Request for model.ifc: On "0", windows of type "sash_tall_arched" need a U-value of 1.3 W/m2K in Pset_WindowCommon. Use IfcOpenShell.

First a look at what the model holds.

```python
import ifcopenshell
import ifcopenshell.util.element

model = ifcopenshell.open("model.ifc")
print(model.schema)
storey = next(s for s in model.by_type("IfcBuildingStorey") if s.Name == "0")
windows = [e for e in ifcopenshell.util.element.get_decomposition(storey) if e.is_a("IfcWindow")]
seen = {}
for e in windows:
    element_type = ifcopenshell.util.element.get_type(e)
    key = (element_type.Name if element_type != e and element_type else None, ifcopenshell.util.element.get_pset(e, "Pset_WindowCommon", "ThermalTransmittance"))
    seen[key] = seen.get(key, 0) + 1
for (name, value), count in sorted(seen.items(), key=str):
    print(count, "x", name, "|", value)
```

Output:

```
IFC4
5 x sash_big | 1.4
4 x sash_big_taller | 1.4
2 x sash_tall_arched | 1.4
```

```python
import ifcopenshell
import ifcopenshell.api.pset
import ifcopenshell.util.element

model = ifcopenshell.open("model.ifc")

storey = next(s for s in model.by_type("IfcBuildingStorey") if s.Name == "0")
windows = [e for e in ifcopenshell.util.element.get_decomposition(storey) if e.is_a("IfcWindow")]

count = 0
for e in windows:
    element_type = ifcopenshell.util.element.get_type(e)
    if element_type in (None, e) or element_type.Name != "sash_tall_arched":
        continue
    # add_pset returns the element's existing set when there is one.
    pset = ifcopenshell.api.pset.add_pset(model, product=e, name="Pset_WindowCommon")
    ifcopenshell.api.pset.edit_pset(model, pset=pset, properties={"ThermalTransmittance": 1.3})
    count += 1

print(count, "windows updated")

model.write("model_v2.ifc")
```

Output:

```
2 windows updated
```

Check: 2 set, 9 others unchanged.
